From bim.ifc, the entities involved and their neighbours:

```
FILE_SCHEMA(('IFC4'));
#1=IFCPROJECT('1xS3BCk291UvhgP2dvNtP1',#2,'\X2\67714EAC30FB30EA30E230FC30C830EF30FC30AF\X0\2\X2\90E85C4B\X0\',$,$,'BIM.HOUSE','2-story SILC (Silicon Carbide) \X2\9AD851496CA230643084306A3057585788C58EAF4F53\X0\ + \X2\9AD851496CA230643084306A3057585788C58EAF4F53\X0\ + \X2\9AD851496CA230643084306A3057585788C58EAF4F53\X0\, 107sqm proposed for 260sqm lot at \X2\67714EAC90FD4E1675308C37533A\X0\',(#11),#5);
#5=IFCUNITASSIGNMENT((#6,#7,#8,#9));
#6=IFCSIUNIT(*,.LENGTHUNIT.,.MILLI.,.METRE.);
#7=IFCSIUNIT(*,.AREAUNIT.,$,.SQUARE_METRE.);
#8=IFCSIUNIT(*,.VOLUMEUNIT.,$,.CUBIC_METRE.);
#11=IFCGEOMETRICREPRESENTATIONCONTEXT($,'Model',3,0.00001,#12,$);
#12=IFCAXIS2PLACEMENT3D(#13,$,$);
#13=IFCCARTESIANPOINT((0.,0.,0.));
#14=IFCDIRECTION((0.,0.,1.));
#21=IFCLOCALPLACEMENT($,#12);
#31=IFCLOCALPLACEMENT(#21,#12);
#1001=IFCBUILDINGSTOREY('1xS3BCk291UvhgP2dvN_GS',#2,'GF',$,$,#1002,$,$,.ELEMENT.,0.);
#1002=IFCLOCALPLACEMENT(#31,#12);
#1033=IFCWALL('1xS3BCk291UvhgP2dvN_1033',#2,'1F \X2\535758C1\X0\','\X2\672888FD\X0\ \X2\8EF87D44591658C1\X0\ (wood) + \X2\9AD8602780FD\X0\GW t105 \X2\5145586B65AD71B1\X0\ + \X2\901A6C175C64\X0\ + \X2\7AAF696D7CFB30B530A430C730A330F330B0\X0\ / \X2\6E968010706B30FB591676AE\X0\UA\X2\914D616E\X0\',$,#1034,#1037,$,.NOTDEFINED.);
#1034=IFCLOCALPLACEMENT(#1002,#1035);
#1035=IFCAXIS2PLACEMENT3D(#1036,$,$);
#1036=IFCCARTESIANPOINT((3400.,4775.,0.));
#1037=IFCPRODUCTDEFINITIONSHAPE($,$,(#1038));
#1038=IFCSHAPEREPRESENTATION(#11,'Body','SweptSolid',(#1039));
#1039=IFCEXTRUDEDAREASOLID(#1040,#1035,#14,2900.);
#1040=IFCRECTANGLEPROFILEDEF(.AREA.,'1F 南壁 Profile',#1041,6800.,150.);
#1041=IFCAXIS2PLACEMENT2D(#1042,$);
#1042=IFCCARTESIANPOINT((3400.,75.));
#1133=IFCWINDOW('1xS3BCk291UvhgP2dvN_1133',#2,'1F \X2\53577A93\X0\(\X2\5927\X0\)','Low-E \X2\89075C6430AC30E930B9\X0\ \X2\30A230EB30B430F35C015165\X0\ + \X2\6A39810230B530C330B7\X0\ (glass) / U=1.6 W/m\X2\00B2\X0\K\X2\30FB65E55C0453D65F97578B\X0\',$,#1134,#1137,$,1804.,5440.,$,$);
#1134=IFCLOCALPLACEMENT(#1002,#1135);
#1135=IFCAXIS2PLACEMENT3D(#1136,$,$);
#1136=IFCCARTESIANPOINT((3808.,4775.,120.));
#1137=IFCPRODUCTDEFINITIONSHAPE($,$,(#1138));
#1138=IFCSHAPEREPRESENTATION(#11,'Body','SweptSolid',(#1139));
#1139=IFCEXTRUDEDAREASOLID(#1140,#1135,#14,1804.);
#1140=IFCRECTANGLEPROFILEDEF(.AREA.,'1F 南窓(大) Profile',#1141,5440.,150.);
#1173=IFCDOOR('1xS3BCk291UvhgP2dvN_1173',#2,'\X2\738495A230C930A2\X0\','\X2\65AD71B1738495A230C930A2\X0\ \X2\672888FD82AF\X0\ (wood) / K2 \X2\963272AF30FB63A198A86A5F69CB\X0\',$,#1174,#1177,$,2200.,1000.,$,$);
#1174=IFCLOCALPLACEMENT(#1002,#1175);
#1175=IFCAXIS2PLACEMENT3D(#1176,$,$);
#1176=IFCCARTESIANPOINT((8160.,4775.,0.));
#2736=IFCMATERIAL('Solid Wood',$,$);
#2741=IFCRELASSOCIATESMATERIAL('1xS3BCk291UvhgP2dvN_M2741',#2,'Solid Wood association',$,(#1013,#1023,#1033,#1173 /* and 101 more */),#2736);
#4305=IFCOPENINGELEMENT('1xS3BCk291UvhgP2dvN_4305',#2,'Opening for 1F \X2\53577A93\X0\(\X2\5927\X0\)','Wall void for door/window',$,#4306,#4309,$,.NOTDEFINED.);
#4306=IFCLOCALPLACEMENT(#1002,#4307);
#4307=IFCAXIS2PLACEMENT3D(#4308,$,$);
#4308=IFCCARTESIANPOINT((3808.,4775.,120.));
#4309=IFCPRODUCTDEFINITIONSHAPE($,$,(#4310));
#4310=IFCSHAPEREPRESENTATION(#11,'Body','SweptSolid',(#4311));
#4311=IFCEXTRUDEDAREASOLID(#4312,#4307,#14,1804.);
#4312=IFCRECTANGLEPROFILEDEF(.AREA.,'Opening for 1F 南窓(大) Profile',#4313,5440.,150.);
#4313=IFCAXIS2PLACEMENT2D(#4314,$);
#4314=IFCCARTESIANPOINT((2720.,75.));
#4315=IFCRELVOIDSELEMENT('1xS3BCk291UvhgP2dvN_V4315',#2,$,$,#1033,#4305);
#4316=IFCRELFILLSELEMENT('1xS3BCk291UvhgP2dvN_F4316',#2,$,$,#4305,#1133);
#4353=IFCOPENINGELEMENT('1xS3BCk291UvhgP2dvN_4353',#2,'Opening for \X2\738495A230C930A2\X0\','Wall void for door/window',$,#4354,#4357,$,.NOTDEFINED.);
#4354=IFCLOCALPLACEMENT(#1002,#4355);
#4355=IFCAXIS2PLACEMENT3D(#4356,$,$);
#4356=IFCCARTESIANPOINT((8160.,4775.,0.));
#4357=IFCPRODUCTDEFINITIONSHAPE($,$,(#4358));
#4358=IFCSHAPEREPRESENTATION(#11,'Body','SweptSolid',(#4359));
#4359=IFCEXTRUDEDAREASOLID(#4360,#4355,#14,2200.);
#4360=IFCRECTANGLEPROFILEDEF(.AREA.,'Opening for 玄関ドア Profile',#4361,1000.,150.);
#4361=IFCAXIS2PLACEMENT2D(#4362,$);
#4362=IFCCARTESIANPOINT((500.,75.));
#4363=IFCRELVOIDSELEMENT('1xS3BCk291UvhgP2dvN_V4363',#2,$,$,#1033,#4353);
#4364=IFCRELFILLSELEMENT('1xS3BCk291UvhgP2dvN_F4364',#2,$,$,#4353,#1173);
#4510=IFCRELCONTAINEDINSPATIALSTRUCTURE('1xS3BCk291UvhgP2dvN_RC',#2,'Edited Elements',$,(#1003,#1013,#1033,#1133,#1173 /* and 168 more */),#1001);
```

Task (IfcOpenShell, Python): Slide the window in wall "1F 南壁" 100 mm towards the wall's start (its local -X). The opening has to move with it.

```python
import ifcopenshell
import ifcopenshell.api.geometry
import ifcopenshell.util.placement

model = ifcopenshell.open("bim.ifc")

window = model.by_guid("1xS3BCk291UvhgP2dvN_1133")
opening = window.FillsVoids[0].RelatingOpeningElement
wall = opening.VoidsElements[0].RelatingBuildingElement

wall_matrix = ifcopenshell.util.placement.get_local_placement(wall.ObjectPlacement)
shift = wall_matrix[:3, 0] * -100.0
before = ifcopenshell.util.placement.get_local_placement(window.ObjectPlacement)[:3, 3].copy()

# The window is not placed relative to its opening, so move both.
for product in (opening, window):
    matrix = ifcopenshell.util.placement.get_local_placement(product.ObjectPlacement)
    matrix[:3, 3] += shift
    ifcopenshell.api.geometry.edit_object_placement(model, product=product, matrix=matrix, is_si=False)

after = ifcopenshell.util.placement.get_local_placement(window.ObjectPlacement)[:3, 3]
print("window moved by", (after - before).round(3) + 0.0)

model.write("bim_rev.ifc")
```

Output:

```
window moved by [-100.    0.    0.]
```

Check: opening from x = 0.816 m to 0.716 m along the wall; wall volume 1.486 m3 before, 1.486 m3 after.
